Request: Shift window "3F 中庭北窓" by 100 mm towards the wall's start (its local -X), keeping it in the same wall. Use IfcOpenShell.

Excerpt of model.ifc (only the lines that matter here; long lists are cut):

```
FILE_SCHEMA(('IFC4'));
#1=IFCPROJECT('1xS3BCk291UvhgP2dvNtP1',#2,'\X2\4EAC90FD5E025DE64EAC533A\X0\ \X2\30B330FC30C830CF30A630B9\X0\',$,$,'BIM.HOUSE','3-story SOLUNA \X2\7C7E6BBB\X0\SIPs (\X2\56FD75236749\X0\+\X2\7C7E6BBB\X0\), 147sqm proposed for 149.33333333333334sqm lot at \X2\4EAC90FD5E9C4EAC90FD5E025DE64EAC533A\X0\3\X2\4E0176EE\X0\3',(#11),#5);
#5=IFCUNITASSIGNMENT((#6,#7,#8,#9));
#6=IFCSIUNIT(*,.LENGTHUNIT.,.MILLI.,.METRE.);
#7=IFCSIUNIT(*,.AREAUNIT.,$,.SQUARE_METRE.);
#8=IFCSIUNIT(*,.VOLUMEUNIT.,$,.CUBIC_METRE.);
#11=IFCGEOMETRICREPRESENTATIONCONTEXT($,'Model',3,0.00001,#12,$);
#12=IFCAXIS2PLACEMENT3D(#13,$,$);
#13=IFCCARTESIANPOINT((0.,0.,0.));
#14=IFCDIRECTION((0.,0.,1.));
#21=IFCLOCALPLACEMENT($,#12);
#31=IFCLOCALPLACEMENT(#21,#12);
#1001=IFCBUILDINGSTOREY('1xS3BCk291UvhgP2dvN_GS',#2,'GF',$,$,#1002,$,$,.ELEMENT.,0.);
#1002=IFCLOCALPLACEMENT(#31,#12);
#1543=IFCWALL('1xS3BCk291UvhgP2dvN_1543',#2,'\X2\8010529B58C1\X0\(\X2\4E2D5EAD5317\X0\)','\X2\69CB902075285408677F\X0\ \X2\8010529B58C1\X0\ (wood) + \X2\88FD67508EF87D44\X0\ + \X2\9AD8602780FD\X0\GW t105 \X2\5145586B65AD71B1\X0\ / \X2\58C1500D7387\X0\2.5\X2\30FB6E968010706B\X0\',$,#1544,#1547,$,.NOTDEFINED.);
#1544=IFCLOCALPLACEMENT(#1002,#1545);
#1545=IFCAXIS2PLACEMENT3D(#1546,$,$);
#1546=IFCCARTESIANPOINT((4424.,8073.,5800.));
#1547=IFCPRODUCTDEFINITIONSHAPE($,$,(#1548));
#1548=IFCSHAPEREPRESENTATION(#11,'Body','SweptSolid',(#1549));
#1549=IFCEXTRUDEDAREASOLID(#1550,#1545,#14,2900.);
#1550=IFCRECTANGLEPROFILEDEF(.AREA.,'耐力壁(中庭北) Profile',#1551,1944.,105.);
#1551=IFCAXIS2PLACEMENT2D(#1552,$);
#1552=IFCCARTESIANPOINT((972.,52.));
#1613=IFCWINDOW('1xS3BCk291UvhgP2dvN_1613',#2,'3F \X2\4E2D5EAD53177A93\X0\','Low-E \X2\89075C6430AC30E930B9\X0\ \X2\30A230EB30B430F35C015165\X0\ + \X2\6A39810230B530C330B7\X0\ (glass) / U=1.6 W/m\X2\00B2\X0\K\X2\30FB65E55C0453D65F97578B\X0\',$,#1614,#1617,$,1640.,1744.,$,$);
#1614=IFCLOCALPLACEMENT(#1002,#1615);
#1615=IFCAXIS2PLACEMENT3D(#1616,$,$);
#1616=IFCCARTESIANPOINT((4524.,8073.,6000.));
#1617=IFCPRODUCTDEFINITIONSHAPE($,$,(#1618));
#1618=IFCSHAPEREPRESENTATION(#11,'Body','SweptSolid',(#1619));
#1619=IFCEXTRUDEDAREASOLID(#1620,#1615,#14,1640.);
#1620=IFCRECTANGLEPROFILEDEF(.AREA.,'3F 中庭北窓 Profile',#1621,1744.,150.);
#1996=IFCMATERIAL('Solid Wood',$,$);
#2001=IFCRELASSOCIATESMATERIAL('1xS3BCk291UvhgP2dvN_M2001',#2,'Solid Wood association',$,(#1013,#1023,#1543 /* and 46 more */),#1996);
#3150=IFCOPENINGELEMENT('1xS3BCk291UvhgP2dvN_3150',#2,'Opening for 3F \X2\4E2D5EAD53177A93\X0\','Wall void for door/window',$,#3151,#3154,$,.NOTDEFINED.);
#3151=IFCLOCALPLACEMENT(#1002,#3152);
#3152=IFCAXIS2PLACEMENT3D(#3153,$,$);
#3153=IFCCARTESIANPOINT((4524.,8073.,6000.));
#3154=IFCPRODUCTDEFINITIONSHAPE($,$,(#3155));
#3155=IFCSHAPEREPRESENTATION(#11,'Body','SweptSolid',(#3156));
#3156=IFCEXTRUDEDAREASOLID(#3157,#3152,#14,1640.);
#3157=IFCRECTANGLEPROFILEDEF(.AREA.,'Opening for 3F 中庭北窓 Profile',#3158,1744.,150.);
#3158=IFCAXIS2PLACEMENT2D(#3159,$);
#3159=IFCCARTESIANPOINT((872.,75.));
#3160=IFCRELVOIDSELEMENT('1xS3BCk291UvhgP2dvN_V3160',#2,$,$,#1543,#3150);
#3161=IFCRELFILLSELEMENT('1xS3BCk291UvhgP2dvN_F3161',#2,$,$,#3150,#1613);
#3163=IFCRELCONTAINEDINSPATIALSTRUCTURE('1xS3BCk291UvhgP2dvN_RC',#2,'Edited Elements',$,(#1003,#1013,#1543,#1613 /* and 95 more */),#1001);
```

```python
import ifcopenshell
import ifcopenshell.api.geometry
import ifcopenshell.util.placement

model = ifcopenshell.open("model.ifc")

window = model.by_guid("1xS3BCk291UvhgP2dvN_1613")
opening = window.FillsVoids[0].RelatingOpeningElement
wall = opening.VoidsElements[0].RelatingBuildingElement

wall_matrix = ifcopenshell.util.placement.get_local_placement(wall.ObjectPlacement)
shift = wall_matrix[:3, 0] * -100.0
before = ifcopenshell.util.placement.get_local_placement(window.ObjectPlacement)[:3, 3].copy()

# The window is not placed relative to its opening, so move both.
for product in (opening, window):
    matrix = ifcopenshell.util.placement.get_local_placement(product.ObjectPlacement)
    matrix[:3, 3] += shift
    ifcopenshell.api.geometry.edit_object_placement(model, product=product, matrix=matrix, is_si=False)

after = ifcopenshell.util.placement.get_local_placement(window.ObjectPlacement)[:3, 3]
print("window moved by", (after - before).round(3) + 0.0)

model.write("model-out.ifc")
```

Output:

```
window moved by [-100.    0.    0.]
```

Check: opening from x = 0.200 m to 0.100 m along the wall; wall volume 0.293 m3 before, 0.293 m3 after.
